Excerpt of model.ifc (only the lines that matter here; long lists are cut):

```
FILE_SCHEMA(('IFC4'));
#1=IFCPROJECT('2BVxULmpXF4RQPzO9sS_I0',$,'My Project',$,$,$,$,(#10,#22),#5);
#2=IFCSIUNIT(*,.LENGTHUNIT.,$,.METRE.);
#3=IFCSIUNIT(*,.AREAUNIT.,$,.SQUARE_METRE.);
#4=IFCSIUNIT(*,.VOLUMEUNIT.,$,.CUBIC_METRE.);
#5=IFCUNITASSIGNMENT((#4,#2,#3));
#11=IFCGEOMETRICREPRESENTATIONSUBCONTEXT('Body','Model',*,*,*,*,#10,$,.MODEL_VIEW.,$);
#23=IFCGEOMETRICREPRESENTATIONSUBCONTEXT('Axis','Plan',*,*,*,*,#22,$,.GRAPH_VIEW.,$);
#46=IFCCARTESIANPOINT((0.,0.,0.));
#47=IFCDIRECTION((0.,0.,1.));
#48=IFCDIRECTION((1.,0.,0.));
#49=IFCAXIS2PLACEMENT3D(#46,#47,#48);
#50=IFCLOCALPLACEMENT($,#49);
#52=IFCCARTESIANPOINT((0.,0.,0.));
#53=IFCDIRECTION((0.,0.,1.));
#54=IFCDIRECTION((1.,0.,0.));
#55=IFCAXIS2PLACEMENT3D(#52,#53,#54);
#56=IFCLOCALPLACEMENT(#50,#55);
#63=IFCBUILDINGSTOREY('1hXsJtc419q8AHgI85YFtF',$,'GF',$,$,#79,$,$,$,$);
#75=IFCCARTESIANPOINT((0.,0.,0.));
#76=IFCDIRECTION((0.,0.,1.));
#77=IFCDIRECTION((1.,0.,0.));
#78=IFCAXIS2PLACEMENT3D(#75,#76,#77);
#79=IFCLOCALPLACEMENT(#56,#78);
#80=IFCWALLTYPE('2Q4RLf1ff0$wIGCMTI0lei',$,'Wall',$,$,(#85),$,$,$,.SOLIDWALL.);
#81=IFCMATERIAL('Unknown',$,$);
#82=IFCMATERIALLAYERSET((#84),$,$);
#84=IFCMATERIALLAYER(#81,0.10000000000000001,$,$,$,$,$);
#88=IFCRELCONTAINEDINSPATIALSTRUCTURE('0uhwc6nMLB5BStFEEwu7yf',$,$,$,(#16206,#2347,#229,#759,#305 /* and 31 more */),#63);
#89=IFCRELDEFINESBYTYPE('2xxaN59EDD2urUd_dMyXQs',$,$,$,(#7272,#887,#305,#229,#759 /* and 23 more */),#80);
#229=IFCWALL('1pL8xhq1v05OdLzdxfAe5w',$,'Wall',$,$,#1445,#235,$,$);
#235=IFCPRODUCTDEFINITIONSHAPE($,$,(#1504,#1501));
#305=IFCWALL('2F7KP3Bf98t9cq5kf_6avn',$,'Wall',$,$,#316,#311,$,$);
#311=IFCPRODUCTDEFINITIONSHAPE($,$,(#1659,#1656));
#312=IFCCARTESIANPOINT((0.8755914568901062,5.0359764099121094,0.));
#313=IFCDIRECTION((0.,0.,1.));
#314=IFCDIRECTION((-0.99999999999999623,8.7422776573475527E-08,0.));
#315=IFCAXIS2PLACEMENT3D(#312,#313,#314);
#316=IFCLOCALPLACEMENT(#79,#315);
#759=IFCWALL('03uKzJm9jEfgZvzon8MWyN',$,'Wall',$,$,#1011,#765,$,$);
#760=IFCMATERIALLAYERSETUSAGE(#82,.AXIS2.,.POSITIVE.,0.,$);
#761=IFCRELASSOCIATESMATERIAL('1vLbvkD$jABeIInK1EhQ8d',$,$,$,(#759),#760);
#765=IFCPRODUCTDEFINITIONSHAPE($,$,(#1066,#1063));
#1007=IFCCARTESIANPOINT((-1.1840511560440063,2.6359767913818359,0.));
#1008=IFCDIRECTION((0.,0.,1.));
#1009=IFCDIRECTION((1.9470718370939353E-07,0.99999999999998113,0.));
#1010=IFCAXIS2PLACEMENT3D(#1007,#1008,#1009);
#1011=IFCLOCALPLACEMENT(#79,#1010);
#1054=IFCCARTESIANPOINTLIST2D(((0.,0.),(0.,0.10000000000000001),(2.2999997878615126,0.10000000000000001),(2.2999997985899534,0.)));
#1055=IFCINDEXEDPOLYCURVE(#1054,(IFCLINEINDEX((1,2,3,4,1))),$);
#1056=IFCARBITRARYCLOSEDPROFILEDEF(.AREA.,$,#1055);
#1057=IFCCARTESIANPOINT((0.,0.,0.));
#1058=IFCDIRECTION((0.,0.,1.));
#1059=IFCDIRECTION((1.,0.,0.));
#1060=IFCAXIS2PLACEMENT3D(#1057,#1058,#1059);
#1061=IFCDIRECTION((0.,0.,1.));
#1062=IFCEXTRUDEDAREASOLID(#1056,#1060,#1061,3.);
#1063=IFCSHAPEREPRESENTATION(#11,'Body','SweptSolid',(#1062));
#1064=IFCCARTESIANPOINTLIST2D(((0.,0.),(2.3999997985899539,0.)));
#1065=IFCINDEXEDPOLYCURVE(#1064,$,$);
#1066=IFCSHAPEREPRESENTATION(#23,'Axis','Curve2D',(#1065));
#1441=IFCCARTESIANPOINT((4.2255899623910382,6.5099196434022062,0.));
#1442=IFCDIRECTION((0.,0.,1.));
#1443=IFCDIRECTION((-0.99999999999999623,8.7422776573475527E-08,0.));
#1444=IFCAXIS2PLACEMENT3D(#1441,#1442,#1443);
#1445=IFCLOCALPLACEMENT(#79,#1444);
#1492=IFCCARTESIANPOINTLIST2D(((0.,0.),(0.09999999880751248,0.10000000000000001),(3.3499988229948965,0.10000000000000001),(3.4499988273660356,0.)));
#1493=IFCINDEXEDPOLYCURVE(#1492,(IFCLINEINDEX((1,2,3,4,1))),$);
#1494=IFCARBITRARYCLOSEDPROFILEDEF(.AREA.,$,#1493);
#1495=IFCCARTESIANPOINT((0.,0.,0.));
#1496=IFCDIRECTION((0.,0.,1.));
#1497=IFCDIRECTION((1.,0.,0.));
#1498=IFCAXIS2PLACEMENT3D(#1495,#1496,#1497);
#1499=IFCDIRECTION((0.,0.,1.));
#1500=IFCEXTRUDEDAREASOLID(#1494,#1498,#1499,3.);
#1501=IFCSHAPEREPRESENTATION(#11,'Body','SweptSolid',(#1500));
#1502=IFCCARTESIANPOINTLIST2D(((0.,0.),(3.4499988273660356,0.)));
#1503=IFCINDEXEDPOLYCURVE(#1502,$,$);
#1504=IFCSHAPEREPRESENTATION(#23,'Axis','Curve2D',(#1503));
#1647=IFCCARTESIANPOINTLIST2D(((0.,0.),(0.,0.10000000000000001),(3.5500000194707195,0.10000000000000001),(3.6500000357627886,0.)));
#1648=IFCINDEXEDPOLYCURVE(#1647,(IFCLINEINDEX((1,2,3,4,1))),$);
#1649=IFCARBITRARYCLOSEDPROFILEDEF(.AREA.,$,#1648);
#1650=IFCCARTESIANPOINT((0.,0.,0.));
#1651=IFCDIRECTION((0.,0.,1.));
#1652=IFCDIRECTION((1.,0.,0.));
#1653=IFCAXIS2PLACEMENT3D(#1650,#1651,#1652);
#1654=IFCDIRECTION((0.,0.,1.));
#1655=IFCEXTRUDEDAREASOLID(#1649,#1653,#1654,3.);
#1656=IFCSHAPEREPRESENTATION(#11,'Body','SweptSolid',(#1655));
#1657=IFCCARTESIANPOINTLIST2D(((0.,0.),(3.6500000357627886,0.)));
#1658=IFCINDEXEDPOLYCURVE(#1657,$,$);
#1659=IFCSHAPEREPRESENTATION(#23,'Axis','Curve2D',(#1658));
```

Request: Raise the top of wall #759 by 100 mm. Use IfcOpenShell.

```python
import ifcopenshell
import ifcopenshell.geom
import ifcopenshell.util.representation
import ifcopenshell.util.shape

model = ifcopenshell.open("model.ifc")
settings = ifcopenshell.geom.settings()


def volume(element):
    """Net volume in cubic metres, openings subtracted."""
    shape = ifcopenshell.geom.create_shape(settings, element)
    return ifcopenshell.util.shape.get_volume(shape.geometry)


wall = model.by_guid("03uKzJm9jEfgZvzon8MWyN")
before = volume(wall)

body = ifcopenshell.util.representation.get_representation(wall, "Model", "Body")
solid = body.Items[0]
old_height = solid.Depth
solid.Depth += 0.1
after = volume(wall)

print(f"height {old_height:g} -> {solid.Depth:g}, volume {before:.3f} -> {after:.3f} m3")

model.write("model_edited.ifc")
```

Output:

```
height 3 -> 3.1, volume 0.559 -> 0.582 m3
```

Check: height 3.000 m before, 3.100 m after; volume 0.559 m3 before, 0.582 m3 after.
